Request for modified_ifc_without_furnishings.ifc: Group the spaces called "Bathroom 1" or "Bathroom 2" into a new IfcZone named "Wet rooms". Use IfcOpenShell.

First a look at what the model holds.

```python
import ifcopenshell

model = ifcopenshell.open("modified_ifc_without_furnishings.ifc")
print(model.schema)
seen = {}
for space in model.by_type("IfcSpace"):
    seen[space.LongName] = seen.get(space.LongName, 0) + 1
for name, count in sorted(seen.items(), key=str):
    print(count, "x", name)
print("zones:", [z.Name for z in model.by_type("IfcZone")][:20])
```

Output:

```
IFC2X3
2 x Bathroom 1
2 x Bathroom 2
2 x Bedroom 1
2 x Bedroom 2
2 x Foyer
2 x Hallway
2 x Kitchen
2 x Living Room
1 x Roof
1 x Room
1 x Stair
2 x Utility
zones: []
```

```python
import ifcopenshell
import ifcopenshell.api.group
import ifcopenshell.api.root

model = ifcopenshell.open("modified_ifc_without_furnishings.ifc")

names = {"Bathroom 1", "Bathroom 2"}
spaces = [s for s in model.by_type("IfcSpace") if s.LongName in names]

zone = ifcopenshell.api.root.create_entity(model, ifc_class="IfcZone", name="Wet rooms")
ifcopenshell.api.group.assign_group(model, products=spaces, group=zone)
print(len(spaces), "spaces in", zone.Name)

model.write("modified_ifc_without_furnishings_rev.ifc")
```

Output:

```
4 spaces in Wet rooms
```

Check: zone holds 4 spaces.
